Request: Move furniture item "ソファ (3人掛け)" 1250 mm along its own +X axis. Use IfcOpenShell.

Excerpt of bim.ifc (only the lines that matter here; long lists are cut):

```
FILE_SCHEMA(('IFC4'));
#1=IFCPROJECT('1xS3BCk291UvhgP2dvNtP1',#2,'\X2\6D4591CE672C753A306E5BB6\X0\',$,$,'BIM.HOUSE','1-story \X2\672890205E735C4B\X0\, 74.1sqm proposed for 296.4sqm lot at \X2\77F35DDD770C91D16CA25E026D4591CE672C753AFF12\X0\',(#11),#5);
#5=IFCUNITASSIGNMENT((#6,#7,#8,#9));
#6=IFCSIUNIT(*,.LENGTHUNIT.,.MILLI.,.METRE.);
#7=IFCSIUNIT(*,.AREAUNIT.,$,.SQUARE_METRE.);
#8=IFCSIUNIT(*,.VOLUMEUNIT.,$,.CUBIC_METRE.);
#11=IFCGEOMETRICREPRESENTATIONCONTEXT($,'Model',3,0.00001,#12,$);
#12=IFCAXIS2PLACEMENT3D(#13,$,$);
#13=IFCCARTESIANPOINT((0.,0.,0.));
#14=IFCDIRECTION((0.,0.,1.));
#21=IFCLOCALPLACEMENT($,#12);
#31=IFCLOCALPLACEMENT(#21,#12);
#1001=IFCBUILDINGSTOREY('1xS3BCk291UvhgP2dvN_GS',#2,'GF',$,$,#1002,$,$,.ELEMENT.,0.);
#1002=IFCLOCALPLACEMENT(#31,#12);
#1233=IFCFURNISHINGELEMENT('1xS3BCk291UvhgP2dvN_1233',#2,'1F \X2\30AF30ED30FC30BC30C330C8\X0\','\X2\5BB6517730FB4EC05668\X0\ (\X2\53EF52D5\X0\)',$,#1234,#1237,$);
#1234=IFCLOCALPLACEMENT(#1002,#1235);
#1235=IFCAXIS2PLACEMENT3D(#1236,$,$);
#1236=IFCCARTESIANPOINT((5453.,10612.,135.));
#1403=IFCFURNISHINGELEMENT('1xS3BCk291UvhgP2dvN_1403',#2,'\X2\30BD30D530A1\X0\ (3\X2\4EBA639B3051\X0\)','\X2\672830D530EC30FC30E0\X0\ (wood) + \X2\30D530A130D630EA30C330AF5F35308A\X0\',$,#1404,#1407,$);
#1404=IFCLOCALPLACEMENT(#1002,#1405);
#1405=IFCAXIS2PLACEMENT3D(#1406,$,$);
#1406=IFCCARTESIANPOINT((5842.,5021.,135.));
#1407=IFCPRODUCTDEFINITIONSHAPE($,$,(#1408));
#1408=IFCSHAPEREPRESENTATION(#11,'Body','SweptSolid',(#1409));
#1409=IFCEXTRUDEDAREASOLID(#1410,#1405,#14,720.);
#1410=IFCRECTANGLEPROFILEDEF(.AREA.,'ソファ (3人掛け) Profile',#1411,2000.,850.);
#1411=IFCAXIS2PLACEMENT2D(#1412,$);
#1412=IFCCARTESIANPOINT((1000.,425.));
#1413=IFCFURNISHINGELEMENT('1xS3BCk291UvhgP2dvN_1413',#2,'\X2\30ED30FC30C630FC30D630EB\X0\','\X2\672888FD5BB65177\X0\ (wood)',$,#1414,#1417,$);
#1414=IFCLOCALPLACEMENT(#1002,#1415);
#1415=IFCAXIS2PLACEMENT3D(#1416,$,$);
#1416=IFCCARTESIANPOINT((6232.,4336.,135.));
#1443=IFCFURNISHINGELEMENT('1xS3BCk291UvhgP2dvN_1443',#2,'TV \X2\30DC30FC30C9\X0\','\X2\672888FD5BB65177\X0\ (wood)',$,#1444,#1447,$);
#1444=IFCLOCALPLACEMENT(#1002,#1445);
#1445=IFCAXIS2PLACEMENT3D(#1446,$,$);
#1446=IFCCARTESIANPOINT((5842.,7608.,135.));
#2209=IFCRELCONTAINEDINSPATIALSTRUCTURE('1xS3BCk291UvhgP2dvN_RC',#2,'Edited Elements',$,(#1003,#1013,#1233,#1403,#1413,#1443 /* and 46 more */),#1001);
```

```python
import ifcopenshell
import ifcopenshell.api.geometry
import ifcopenshell.util.placement

model = ifcopenshell.open("bim.ifc")

item = model.by_id(1403)
matrix = ifcopenshell.util.placement.get_local_placement(item.ObjectPlacement)
matrix[:3, 3] += matrix[:3, 0] * 1250.0
ifcopenshell.api.geometry.edit_object_placement(model, product=item, matrix=matrix, is_si=False)

print(ifcopenshell.util.placement.get_local_placement(item.ObjectPlacement).round(3) + 0.0)

model.write("bim_edited.ifc")
```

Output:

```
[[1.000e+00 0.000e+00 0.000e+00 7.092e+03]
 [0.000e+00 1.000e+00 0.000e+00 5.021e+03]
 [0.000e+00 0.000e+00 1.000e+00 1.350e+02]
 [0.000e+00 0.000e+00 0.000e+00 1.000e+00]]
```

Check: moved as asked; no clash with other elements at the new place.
